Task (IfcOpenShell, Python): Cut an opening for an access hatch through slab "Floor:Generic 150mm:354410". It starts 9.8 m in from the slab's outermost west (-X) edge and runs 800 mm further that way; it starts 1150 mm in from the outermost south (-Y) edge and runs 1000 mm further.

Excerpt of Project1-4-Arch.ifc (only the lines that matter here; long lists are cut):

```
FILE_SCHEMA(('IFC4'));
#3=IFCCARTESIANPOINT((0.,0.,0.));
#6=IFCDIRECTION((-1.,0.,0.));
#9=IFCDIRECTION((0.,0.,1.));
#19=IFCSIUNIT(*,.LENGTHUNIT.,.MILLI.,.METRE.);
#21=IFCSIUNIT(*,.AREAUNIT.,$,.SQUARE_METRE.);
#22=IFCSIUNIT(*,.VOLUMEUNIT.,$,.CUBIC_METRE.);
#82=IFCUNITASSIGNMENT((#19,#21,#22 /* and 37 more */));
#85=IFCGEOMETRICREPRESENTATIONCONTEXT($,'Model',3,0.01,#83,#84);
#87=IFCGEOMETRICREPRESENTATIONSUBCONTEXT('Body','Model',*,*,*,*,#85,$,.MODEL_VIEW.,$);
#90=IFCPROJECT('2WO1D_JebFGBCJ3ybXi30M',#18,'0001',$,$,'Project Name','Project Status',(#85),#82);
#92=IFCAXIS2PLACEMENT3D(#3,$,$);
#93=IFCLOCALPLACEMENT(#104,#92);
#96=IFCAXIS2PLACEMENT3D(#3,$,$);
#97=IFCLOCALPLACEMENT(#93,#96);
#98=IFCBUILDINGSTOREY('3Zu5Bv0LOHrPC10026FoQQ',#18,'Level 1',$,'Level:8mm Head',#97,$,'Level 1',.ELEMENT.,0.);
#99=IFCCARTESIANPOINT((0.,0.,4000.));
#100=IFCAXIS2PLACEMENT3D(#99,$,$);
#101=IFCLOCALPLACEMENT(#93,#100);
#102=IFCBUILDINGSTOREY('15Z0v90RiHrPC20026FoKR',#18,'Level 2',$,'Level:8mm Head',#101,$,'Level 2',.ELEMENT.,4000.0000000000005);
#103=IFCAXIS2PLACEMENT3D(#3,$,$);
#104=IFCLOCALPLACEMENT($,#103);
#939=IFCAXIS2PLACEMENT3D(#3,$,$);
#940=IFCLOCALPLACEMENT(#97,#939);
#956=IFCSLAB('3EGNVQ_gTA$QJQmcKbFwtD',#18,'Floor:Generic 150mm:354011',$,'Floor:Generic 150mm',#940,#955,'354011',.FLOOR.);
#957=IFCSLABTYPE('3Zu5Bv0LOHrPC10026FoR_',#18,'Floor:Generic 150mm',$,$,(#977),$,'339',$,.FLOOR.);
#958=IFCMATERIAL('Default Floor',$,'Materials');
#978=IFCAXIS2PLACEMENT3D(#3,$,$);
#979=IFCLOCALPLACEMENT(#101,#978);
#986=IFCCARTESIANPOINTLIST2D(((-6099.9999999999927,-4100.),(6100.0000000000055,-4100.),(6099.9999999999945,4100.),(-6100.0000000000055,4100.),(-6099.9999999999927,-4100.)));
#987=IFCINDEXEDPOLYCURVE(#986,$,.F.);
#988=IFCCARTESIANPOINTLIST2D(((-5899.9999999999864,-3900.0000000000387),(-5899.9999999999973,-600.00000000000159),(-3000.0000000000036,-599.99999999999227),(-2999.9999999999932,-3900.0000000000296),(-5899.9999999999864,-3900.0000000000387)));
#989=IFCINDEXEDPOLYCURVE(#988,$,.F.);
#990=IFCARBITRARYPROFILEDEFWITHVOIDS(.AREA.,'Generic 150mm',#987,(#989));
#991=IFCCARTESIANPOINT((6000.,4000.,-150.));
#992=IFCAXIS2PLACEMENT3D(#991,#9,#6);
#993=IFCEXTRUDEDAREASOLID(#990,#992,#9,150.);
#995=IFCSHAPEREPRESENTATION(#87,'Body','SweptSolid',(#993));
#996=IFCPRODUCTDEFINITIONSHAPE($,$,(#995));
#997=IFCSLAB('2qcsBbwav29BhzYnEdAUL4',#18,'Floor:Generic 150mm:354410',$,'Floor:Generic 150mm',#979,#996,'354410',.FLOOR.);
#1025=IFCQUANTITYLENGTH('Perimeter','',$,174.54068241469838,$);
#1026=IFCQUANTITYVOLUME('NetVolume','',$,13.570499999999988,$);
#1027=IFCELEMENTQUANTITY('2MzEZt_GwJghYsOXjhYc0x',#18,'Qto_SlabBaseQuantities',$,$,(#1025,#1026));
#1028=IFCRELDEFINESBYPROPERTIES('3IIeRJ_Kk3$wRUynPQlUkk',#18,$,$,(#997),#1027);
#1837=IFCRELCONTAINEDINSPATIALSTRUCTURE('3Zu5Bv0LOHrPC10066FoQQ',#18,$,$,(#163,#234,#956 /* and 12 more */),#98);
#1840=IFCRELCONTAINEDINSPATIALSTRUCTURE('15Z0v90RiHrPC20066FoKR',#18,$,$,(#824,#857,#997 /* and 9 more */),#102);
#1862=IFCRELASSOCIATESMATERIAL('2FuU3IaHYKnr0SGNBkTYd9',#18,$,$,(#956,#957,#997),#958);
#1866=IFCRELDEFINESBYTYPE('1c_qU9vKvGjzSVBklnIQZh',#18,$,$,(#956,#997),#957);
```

```python
import numpy as np
import ifcopenshell
import ifcopenshell.api.feature
import ifcopenshell.api.geometry
import ifcopenshell.api.pset
import ifcopenshell.api.root
import ifcopenshell.geom
import ifcopenshell.util.element
import ifcopenshell.util.placement
import ifcopenshell.util.representation
import ifcopenshell.util.shape
import ifcopenshell.util.unit

model = ifcopenshell.open("Project1-4-Arch.ifc")
unit_scale = ifcopenshell.util.unit.calculate_unit_scale(model)
volume_scale = ifcopenshell.util.unit.calculate_unit_scale(model, "VOLUMEUNIT")
settings = ifcopenshell.geom.settings()


def volume(element):
    """Net volume in cubic metres, openings subtracted."""
    shape = ifcopenshell.geom.create_shape(settings, element)
    return ifcopenshell.util.shape.get_volume(shape.geometry)


slab = model.by_id(997)
before = volume(slab)

# Extent in the slab's own axes, in metres. The edges named are its -X and -Y sides.
slab_shape = ifcopenshell.geom.create_shape(settings, slab)
vertices = ifcopenshell.util.shape.get_vertices(slab_shape.geometry)
x_min, y_min, bottom = vertices.min(axis=0)
top = vertices[:, 2].max()

opening = ifcopenshell.api.root.create_entity(model, ifc_class="IfcOpeningElement", name="Access hatch opening", predefined_type="OPENING")
context = ifcopenshell.util.representation.get_context(model, "Model", "Body", "MODEL_VIEW")
width, depth = 0.8, 1
outline = [(0.0, 0.0), (width, 0.0), (width, depth), (0.0, depth), (0.0, 0.0)]
# Overshoot both faces by 50 mm so the cut is clean.
shape = ifcopenshell.api.geometry.add_slab_representation(
    model, context=context, depth=top - bottom + 0.1, polyline=outline
)
ifcopenshell.api.geometry.assign_representation(model, product=opening, representation=shape)

matrix = ifcopenshell.util.placement.get_local_placement(slab.ObjectPlacement)
matrix[:, 3] = matrix @ np.append(np.array([x_min + 9.8, y_min + 1.15, bottom - 0.05]) / unit_scale, 1.0)
ifcopenshell.api.geometry.edit_object_placement(model, product=opening, matrix=matrix, is_si=False)
ifcopenshell.api.feature.add_feature(model, feature=opening, element=slab)

after = volume(slab)

# Update the slab's stored quantities.
qto = model.by_id(ifcopenshell.util.element.get_pset(slab, "Qto_SlabBaseQuantities", should_inherit=False)["id"])
ifcopenshell.api.pset.edit_qto(model, qto=qto, properties={"NetVolume": after / volume_scale})

print(f"slab volume {before:.3f} -> {after:.3f} m3")

model.write("Project1-4-Arch-out.ifc")
```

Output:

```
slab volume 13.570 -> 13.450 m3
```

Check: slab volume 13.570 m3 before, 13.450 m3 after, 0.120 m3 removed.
